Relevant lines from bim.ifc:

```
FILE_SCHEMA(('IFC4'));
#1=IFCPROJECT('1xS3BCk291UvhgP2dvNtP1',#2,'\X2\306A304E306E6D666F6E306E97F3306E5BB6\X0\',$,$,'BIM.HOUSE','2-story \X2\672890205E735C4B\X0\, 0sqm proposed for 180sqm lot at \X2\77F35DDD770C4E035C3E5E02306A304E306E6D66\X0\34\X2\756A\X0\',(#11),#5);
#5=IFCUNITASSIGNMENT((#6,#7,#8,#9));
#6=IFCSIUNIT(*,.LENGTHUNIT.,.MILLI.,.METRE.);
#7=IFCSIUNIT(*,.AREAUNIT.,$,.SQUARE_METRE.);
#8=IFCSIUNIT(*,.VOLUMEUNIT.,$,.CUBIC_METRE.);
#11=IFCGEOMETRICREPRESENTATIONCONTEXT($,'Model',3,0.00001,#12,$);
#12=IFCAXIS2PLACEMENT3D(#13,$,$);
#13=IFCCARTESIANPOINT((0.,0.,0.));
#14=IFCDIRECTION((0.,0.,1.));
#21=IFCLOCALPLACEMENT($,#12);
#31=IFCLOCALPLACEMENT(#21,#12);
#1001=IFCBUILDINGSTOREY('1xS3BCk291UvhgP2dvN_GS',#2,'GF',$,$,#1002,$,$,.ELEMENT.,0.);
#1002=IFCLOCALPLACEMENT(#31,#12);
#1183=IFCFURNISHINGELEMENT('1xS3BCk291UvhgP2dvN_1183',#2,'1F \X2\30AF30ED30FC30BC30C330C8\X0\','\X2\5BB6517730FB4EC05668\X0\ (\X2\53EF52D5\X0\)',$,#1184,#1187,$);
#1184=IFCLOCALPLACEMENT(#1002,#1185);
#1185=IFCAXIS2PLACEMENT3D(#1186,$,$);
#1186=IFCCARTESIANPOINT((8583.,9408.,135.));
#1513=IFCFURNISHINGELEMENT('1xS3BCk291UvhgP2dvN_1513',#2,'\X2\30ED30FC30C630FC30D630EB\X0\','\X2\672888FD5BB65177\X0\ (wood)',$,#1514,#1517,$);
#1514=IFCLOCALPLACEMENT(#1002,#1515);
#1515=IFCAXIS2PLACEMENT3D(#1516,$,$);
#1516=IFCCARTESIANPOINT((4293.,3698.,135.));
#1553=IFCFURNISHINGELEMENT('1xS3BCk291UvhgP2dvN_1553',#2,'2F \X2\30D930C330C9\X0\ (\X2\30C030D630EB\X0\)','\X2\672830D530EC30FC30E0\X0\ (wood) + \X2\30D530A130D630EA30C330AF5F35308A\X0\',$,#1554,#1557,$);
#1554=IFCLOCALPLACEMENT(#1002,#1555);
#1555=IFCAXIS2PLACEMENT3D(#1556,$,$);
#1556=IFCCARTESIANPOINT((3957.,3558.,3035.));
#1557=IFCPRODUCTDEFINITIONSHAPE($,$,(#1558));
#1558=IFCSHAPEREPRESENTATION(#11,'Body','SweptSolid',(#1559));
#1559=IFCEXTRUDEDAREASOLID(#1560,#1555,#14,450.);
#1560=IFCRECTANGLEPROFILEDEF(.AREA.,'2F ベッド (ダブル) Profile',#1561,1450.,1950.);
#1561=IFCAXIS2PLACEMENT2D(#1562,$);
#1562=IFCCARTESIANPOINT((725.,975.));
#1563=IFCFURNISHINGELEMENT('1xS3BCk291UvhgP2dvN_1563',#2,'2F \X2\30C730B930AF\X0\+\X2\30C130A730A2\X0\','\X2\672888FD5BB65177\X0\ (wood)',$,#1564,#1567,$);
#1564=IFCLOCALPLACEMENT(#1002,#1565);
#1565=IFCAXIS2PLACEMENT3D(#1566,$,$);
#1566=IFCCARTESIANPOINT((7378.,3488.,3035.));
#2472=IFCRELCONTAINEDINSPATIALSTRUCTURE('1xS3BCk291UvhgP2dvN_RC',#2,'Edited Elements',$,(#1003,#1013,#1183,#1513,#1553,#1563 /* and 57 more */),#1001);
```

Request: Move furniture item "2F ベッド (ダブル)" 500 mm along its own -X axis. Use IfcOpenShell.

```python
import ifcopenshell
import ifcopenshell.api.geometry
import ifcopenshell.util.placement
import ifcopenshell.util.unit

model = ifcopenshell.open("bim.ifc")
unit_scale = ifcopenshell.util.unit.calculate_unit_scale(model)

item = model.by_id(1553)
matrix = ifcopenshell.util.placement.get_local_placement(item.ObjectPlacement)
matrix[:3, 3] -= matrix[:3, 0] * 0.5 / unit_scale
ifcopenshell.api.geometry.edit_object_placement(model, product=item, matrix=matrix, is_si=False)

print(ifcopenshell.util.placement.get_local_placement(item.ObjectPlacement).round(3) + 0.0)

model.write("bim_updated.ifc")
```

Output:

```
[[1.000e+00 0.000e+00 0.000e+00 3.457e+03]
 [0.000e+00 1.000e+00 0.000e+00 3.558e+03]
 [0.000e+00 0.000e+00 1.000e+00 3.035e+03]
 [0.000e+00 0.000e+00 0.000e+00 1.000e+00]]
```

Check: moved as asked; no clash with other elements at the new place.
